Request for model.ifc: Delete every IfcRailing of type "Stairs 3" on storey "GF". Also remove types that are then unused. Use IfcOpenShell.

First a look at what the model holds.

```python
import ifcopenshell
import ifcopenshell.util.element

model = ifcopenshell.open("model.ifc")
print(model.schema)
storey = next(s for s in model.by_type("IfcBuildingStorey") if s.Name == "GF")
railings = [e for e in ifcopenshell.util.element.get_decomposition(storey) if e.is_a("IfcRailing")]
seen = {}
for e in railings:
    element_type = ifcopenshell.util.element.get_type(e)
    name = element_type.Name if element_type not in (None, e) else None
    seen[name] = seen.get(name, 0) + 1
for name, count in sorted(seen.items(), key=str):
    print(count, "x", name)
```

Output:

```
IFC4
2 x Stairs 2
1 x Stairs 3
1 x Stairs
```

```python
import ifcopenshell
import ifcopenshell.api.root
import ifcopenshell.util.element

model = ifcopenshell.open("model.ifc")

storey = next(s for s in model.by_type("IfcBuildingStorey") if s.Name == "GF")
railings = [e for e in ifcopenshell.util.element.get_decomposition(storey) if e.is_a("IfcRailing")]
targets = [e for e in railings if (t := ifcopenshell.util.element.get_type(e)) not in (None, e) and t.Name == "Stairs 3"]
types = {ifcopenshell.util.element.get_type(e) for e in targets} - {None, *targets}

for e in targets:
    ifcopenshell.api.root.remove_product(model, product=e)
print(len(targets), "removed")

unused = [t for t in types if not ifcopenshell.util.element.get_types(t)]
for t in unused:
    ifcopenshell.api.root.remove_product(model, product=t)
print(len(unused), "unused types removed")

model.write("model_updated.ifc")
```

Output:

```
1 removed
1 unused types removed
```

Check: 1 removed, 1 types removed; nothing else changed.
